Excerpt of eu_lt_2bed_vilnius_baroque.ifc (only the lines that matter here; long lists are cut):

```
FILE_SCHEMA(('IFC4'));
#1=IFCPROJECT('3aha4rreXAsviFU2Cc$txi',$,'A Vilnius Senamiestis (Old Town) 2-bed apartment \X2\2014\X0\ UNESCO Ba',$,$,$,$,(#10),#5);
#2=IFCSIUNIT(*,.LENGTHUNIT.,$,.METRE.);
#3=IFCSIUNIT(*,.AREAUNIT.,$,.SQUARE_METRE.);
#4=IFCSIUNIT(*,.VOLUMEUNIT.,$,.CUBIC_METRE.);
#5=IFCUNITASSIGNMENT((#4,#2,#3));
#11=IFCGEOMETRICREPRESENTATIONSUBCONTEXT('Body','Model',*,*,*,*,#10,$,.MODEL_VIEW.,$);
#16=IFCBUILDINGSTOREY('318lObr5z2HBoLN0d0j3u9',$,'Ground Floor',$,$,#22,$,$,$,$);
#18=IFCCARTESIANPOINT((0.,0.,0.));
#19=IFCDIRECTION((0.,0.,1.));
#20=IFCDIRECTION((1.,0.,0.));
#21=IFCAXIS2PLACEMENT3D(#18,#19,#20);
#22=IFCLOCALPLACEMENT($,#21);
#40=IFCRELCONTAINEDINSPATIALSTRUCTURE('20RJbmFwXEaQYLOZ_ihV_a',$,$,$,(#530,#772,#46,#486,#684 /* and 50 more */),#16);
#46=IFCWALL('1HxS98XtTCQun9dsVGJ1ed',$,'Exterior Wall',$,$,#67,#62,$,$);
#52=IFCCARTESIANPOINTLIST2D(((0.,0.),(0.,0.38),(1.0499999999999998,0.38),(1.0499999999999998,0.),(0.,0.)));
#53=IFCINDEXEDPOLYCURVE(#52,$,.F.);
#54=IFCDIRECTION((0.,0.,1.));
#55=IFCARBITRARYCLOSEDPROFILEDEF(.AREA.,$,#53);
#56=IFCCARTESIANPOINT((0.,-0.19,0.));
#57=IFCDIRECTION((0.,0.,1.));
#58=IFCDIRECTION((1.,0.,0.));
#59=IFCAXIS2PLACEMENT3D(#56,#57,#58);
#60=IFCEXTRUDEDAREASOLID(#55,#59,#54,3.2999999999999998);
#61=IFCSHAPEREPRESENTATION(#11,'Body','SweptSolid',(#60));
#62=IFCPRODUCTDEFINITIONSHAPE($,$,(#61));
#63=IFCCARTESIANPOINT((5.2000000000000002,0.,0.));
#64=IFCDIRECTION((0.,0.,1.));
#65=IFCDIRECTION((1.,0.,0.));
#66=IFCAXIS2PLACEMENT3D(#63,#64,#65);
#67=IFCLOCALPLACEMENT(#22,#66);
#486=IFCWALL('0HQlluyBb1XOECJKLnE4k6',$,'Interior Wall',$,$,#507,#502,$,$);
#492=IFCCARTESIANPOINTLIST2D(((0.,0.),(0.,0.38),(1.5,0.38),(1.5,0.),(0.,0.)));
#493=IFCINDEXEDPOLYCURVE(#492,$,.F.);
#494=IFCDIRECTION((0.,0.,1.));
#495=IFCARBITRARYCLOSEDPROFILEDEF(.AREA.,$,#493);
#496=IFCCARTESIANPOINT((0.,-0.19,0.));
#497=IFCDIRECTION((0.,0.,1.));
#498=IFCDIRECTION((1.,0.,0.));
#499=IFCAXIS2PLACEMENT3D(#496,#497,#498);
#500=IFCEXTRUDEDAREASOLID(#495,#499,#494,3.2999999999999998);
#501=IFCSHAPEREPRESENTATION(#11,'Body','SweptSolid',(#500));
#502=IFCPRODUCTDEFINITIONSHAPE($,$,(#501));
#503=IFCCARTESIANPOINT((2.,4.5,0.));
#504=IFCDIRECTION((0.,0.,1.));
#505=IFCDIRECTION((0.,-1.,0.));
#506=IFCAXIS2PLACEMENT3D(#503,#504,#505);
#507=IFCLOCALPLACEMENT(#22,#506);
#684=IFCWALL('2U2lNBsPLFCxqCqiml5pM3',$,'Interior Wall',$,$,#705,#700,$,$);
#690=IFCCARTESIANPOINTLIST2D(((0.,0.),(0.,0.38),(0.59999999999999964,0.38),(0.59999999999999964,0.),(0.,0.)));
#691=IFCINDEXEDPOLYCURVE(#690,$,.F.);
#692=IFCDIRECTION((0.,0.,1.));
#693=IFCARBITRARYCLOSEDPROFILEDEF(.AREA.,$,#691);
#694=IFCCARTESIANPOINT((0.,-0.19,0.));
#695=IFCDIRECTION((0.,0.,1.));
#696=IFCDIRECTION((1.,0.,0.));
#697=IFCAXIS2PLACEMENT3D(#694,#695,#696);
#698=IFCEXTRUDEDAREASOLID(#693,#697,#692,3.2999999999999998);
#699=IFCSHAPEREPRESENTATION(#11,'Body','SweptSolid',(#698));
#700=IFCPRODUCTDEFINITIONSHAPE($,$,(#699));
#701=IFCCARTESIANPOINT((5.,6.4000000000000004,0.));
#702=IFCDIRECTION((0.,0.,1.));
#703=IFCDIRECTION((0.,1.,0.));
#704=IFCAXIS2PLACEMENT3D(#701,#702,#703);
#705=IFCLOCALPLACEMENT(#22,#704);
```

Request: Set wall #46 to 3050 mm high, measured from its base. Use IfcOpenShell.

```python
import ifcopenshell
import ifcopenshell.geom
import ifcopenshell.util.representation
import ifcopenshell.util.shape
import ifcopenshell.util.unit

model = ifcopenshell.open("eu_lt_2bed_vilnius_baroque.ifc")
unit_scale = ifcopenshell.util.unit.calculate_unit_scale(model)
settings = ifcopenshell.geom.settings()


def volume(element):
    """Net volume in cubic metres, openings subtracted."""
    shape = ifcopenshell.geom.create_shape(settings, element)
    return ifcopenshell.util.shape.get_volume(shape.geometry)


wall = model.by_guid("1HxS98XtTCQun9dsVGJ1ed")
before = volume(wall)

body = ifcopenshell.util.representation.get_representation(wall, "Model", "Body")
solid = body.Items[0]
old_height = solid.Depth
solid.Depth = 3.05 / unit_scale
after = volume(wall)

print(f"height {old_height:g} -> {solid.Depth:g}, volume {before:.3f} -> {after:.3f} m3")

model.write("eu_lt_2bed_vilnius_baroque_edited.ifc")
```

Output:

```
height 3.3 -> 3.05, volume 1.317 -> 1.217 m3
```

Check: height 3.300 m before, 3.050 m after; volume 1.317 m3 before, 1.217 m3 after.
